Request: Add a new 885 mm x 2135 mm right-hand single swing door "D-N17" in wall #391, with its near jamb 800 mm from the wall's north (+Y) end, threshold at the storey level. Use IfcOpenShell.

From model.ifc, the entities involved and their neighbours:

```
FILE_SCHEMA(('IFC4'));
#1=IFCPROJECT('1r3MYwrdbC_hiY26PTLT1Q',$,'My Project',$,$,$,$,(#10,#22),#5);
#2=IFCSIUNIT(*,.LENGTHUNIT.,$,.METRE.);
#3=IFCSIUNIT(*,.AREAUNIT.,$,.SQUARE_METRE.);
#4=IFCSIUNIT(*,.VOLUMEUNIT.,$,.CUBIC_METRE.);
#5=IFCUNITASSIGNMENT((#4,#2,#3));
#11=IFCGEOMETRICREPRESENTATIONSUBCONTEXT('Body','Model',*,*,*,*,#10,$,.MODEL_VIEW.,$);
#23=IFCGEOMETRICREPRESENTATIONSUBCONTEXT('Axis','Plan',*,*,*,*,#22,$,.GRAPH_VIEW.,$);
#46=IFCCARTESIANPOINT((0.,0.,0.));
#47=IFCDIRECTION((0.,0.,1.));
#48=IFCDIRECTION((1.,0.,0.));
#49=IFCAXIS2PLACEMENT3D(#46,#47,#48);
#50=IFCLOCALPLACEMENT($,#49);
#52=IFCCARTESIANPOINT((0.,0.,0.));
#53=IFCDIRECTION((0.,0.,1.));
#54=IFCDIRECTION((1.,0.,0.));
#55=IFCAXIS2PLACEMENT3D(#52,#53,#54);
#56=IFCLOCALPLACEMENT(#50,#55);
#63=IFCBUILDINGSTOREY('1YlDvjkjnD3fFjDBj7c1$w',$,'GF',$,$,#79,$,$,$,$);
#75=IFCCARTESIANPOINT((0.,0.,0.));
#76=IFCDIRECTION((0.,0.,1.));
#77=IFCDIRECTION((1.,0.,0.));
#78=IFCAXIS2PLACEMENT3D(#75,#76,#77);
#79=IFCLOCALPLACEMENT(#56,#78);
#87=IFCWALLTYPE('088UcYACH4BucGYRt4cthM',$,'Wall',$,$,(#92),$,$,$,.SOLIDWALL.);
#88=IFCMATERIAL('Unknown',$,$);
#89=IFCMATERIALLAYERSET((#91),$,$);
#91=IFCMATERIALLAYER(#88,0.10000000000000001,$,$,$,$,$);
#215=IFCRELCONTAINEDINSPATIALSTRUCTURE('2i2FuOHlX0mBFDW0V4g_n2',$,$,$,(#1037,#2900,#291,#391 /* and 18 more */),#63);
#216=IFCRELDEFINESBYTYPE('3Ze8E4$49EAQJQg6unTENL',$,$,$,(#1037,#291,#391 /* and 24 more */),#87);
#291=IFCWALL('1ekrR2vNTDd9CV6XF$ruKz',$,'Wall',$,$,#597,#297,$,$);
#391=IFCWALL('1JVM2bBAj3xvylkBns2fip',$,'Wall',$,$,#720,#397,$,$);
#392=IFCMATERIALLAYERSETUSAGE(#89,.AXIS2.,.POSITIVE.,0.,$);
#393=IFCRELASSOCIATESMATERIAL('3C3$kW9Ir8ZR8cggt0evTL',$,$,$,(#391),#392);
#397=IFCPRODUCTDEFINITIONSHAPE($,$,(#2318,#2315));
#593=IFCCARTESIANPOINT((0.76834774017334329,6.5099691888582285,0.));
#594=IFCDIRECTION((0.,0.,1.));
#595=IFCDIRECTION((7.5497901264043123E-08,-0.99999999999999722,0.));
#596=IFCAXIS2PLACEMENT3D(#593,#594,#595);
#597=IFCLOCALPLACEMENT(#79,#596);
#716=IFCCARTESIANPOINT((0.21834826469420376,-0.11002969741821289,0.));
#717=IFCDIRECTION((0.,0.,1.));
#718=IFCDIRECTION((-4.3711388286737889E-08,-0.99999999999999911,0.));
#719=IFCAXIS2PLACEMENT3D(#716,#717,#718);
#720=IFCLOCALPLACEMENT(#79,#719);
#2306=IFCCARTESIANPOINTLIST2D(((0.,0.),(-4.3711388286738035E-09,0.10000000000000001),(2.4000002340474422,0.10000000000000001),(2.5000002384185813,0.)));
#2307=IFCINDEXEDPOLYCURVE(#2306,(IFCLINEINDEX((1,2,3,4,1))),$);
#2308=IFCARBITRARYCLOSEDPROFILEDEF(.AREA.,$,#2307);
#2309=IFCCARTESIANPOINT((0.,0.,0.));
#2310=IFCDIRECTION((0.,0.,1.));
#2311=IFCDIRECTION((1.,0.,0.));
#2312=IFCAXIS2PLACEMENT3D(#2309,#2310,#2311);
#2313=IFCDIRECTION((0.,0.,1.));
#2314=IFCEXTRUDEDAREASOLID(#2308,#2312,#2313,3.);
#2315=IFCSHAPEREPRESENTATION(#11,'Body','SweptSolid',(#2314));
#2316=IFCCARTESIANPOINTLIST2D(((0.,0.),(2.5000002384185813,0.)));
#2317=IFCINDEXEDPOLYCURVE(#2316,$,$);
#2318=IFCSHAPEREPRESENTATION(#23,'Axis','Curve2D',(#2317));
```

```python
import numpy as np
import ifcopenshell
import ifcopenshell.api.feature
import ifcopenshell.api.geometry
import ifcopenshell.api.root
import ifcopenshell.api.spatial
import ifcopenshell.geom
import ifcopenshell.util.element
import ifcopenshell.util.placement
import ifcopenshell.util.representation
import ifcopenshell.util.shape
import ifcopenshell.util.unit

model = ifcopenshell.open("model.ifc")
unit_scale = ifcopenshell.util.unit.calculate_unit_scale(model)
settings = ifcopenshell.geom.settings()


def volume(element):
    """Net volume in cubic metres, openings subtracted."""
    shape = ifcopenshell.geom.create_shape(settings, element)
    return ifcopenshell.util.shape.get_volume(shape.geometry)


wall = model.by_guid("1JVM2bBAj3xvylkBns2fip")
storey = ifcopenshell.util.element.get_container(wall, ifc_class="IfcBuildingStorey")
context = ifcopenshell.util.representation.get_context(model, "Model", "Body", "MODEL_VIEW")
before = volume(wall)

width, height, from_end, sill = 0.885, 2.135, 0.8, 0.0  # metres

# The wall runs along its own X axis, and the end named is its -X end.
wall_shape = ifcopenshell.geom.create_shape(settings, wall)
x, y, z = ifcopenshell.util.shape.get_vertices(wall_shape.geometry).T
start = x.min() + from_end
face, thickness = float(y.min()), float(y.max() - y.min())
wall_matrix = ifcopenshell.util.placement.get_local_placement(wall.ObjectPlacement)
level = ifcopenshell.util.placement.get_local_placement(storey.ObjectPlacement)[2, 3]


def in_wall(x, y):
    """Placement at x, y metres in the wall's axes, at sill height."""
    matrix = wall_matrix.copy()
    matrix[:, 3] = wall_matrix @ np.array([x / unit_scale, y / unit_scale, 0.0, 1.0])
    matrix[2, 3] = level + sill / unit_scale
    return matrix


# Opening: a box that overshoots both wall faces by 50 mm.
opening = ifcopenshell.api.root.create_entity(model, ifc_class="IfcOpeningElement", predefined_type="OPENING")
box = ifcopenshell.api.geometry.add_wall_representation(
    model, context=context, length=width, height=height, thickness=thickness + 0.1
)
ifcopenshell.api.geometry.assign_representation(model, product=opening, representation=box)
ifcopenshell.api.geometry.edit_object_placement(model, product=opening, matrix=in_wall(start, face - 0.05), is_si=False)
ifcopenshell.api.feature.add_feature(model, feature=opening, element=wall)

door = ifcopenshell.api.root.create_entity(model, ifc_class="IfcDoor", name="D-N17", predefined_type="DOOR")
door.OverallWidth, door.OverallHeight = width / unit_scale, height / unit_scale
door.OperationType = "SINGLE_SWING_RIGHT"
body = ifcopenshell.api.geometry.add_door_representation(
    model,
    context=context,
    overall_width=door.OverallWidth,
    overall_height=door.OverallHeight,
    operation_type="SINGLE_SWING_RIGHT",
    lining_properties={"LiningDepth": thickness / unit_scale, "ThresholdDepth": thickness / unit_scale},
)
ifcopenshell.api.geometry.assign_representation(model, product=door, representation=body)
ifcopenshell.api.spatial.assign_container(model, products=[door], relating_structure=storey)
ifcopenshell.api.feature.add_filling(model, opening=opening, element=door)

# The lining spans the wall, so the door starts at the wall face.
ifcopenshell.api.geometry.edit_object_placement(model, product=door, matrix=in_wall(start, face), is_si=False)

after = volume(wall)

print(f"wall volume {before:.3f} -> {after:.3f} m3")

model.write("model_updated.ifc")
```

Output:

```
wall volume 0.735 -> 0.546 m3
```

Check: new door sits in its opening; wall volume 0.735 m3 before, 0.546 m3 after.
